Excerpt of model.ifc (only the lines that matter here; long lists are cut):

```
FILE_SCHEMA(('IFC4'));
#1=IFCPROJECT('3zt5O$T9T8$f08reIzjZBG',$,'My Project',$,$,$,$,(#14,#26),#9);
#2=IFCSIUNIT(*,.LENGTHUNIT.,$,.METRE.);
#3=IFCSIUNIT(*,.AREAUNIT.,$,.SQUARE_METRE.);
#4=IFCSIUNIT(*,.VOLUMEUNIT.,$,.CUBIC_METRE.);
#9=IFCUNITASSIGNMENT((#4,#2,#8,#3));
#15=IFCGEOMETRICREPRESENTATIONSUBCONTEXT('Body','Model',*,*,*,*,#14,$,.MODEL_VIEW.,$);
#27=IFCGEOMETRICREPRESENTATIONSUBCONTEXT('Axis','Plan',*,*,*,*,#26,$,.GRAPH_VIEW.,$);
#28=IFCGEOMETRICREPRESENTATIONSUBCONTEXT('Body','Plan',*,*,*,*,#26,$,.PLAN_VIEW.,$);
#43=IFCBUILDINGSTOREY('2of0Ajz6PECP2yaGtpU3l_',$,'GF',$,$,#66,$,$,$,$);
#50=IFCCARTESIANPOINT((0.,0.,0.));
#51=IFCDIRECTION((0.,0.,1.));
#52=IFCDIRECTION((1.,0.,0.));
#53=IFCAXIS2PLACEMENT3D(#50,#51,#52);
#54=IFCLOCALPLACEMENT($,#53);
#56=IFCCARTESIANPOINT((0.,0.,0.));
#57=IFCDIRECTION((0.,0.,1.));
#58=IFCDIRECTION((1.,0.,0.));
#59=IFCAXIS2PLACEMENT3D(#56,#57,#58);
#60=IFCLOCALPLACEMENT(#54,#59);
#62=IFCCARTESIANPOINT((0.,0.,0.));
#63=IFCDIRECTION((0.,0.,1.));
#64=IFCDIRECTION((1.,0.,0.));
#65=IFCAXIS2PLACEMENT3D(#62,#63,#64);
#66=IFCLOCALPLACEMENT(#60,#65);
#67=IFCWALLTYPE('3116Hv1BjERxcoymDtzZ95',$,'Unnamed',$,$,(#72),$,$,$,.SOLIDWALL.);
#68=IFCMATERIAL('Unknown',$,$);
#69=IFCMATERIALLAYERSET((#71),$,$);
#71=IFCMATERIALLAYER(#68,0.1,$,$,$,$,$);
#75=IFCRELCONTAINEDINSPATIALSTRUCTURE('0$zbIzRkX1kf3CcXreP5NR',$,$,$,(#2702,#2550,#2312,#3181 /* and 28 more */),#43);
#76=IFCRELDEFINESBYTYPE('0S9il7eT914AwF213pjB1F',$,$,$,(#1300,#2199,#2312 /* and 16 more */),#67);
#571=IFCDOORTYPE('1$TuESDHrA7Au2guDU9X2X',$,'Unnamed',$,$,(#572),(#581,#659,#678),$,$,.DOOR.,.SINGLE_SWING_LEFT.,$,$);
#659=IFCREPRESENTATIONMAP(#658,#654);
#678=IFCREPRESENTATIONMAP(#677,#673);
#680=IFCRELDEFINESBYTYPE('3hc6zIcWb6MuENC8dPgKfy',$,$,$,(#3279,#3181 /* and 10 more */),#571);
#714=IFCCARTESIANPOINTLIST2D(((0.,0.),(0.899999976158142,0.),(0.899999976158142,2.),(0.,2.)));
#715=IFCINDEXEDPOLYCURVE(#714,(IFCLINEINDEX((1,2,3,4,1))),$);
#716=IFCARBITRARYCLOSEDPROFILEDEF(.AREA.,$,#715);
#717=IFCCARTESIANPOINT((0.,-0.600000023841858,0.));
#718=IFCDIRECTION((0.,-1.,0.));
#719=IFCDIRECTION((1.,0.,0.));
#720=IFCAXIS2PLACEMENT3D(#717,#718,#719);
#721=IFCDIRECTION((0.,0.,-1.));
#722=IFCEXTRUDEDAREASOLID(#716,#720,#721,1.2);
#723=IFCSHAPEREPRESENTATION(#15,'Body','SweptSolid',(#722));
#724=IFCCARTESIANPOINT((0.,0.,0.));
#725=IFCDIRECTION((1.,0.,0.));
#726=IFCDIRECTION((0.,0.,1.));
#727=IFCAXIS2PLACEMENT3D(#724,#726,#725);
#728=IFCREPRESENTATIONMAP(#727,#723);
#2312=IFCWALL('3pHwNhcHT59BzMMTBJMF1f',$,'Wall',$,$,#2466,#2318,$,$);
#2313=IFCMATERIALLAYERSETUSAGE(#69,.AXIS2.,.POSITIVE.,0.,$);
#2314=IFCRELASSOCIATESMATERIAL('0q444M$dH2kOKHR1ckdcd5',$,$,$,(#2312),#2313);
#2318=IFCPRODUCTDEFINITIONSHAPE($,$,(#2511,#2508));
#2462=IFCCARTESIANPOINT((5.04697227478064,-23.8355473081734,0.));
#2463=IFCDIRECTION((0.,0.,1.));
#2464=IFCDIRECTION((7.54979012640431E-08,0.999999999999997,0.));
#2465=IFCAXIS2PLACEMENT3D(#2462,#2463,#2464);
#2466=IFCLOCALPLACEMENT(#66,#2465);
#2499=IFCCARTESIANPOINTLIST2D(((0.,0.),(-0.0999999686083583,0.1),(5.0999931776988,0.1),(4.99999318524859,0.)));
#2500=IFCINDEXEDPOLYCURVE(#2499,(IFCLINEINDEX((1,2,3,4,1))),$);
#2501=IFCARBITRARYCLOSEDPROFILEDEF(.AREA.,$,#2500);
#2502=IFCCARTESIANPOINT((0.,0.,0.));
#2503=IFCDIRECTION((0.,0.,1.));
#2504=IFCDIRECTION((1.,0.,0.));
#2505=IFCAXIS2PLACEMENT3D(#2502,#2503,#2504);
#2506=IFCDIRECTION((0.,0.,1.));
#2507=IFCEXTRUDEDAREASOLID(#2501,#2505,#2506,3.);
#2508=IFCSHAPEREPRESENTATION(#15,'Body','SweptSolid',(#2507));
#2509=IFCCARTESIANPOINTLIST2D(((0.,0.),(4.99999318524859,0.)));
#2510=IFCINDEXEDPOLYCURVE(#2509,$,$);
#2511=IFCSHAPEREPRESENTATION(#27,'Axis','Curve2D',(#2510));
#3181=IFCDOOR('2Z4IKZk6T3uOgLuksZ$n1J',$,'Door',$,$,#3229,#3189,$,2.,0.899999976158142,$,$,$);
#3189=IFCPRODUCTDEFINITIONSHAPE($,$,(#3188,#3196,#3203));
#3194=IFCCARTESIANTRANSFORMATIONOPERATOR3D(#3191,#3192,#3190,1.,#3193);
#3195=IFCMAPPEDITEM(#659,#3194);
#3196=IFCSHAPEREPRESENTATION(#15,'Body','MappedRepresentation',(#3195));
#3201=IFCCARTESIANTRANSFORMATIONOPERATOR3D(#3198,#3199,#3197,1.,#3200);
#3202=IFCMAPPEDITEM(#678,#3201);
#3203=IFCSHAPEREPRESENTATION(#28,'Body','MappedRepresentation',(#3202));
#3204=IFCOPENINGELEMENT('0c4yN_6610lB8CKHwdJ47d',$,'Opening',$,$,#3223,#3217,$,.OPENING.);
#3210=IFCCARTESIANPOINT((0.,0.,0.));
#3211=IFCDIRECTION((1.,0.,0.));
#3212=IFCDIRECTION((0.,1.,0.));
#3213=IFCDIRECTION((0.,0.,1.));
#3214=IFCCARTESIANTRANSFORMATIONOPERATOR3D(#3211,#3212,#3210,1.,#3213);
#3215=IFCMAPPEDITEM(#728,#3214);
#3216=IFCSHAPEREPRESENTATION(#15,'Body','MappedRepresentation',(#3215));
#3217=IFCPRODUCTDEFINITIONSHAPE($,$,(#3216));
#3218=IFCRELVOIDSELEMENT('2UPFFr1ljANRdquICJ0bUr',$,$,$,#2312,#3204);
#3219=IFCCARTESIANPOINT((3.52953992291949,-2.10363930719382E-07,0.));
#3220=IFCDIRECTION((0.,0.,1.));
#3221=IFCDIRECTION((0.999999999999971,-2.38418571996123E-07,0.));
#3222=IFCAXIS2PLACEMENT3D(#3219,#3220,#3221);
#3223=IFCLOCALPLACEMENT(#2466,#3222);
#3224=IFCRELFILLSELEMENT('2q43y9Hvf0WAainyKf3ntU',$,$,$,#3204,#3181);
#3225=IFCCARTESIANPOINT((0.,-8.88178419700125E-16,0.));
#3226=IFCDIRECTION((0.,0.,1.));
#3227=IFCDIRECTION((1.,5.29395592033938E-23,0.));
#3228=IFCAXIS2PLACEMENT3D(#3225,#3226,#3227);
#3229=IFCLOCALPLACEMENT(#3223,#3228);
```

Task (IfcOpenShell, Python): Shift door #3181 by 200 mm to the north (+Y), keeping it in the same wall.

```python
import ifcopenshell
import ifcopenshell.api.geometry
import ifcopenshell.util.placement

model = ifcopenshell.open("model.ifc")

door = model.by_guid("2Z4IKZk6T3uOgLuksZ$n1J")
opening = door.FillsVoids[0].RelatingOpeningElement
wall = opening.VoidsElements[0].RelatingBuildingElement

wall_matrix = ifcopenshell.util.placement.get_local_placement(wall.ObjectPlacement)
shift = wall_matrix[:3, 0] * 0.2
before = ifcopenshell.util.placement.get_local_placement(door.ObjectPlacement)[:3, 3].copy()

# The door is placed relative to its opening, so it follows when the opening moves.
matrix = ifcopenshell.util.placement.get_local_placement(opening.ObjectPlacement)
matrix[:3, 3] += shift
ifcopenshell.api.geometry.edit_object_placement(
    model, product=opening, matrix=matrix, is_si=False, should_transform_children=True
)

after = ifcopenshell.util.placement.get_local_placement(door.ObjectPlacement)[:3, 3]
print("door moved by", (after - before).round(3) + 0.0)

model.write("model_rev.ifc")
```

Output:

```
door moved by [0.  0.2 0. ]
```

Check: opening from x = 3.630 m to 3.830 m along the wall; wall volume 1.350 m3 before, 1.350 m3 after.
